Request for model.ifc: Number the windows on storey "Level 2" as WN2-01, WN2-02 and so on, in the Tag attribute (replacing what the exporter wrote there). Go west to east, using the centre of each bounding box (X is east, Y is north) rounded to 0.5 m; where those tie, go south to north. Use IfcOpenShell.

First a look at what the model holds.

```python
import ifcopenshell
import ifcopenshell.util.element
import ifcopenshell.util.placement

model = ifcopenshell.open("model.ifc")
print(model.schema)
storey = next(s for s in model.by_type("IfcBuildingStorey") if s.Name == "Level 2")
windows = [e for e in ifcopenshell.util.element.get_decomposition(storey) if e.is_a("IfcWindow")]
for e in sorted(windows, key=lambda e: e.id()):
    origin = ifcopenshell.util.placement.get_local_placement(e.ObjectPlacement)[:3, 3]
    print(e.id(), e.Tag, e.Name, origin.round(2) + 0.0, sep=" | ")
```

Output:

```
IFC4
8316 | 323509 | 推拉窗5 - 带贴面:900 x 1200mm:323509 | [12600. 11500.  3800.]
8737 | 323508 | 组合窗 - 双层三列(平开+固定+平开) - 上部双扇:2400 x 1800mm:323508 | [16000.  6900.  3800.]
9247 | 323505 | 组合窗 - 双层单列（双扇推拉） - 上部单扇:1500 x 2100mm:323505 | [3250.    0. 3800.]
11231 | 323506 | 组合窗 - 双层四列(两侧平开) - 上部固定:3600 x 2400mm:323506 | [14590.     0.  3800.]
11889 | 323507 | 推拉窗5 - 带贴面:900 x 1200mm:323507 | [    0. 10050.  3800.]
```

```python
import ifcopenshell
import ifcopenshell.geom
import ifcopenshell.util.element
import ifcopenshell.util.shape

model = ifcopenshell.open("model.ifc")
settings = ifcopenshell.geom.settings()
settings.set("use-world-coords", True)


def centre(element):
    shape = ifcopenshell.geom.create_shape(settings, element)
    return ifcopenshell.util.shape.get_bbox_centroid(shape.geometry)


storey = next(s for s in model.by_type("IfcBuildingStorey") if s.Name == "Level 2")
windows = [e for e in ifcopenshell.util.element.get_decomposition(storey) if e.is_a("IfcWindow")]

# Insertion points can sit at a corner or the storey origin, so sort by the geometry (in metres).
centres = {e: centre(e) for e in windows}
windows.sort(key=lambda e: (round(centres[e][0] / 0.5), centres[e][1]))

for i, e in enumerate(windows, start=1):
    number = f"WN2-{i:02d}"
    e.Tag = number
    print(e.id(), number)

model.write("model_edited.ifc")
```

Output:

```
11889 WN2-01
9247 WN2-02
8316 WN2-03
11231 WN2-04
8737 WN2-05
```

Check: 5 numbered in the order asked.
